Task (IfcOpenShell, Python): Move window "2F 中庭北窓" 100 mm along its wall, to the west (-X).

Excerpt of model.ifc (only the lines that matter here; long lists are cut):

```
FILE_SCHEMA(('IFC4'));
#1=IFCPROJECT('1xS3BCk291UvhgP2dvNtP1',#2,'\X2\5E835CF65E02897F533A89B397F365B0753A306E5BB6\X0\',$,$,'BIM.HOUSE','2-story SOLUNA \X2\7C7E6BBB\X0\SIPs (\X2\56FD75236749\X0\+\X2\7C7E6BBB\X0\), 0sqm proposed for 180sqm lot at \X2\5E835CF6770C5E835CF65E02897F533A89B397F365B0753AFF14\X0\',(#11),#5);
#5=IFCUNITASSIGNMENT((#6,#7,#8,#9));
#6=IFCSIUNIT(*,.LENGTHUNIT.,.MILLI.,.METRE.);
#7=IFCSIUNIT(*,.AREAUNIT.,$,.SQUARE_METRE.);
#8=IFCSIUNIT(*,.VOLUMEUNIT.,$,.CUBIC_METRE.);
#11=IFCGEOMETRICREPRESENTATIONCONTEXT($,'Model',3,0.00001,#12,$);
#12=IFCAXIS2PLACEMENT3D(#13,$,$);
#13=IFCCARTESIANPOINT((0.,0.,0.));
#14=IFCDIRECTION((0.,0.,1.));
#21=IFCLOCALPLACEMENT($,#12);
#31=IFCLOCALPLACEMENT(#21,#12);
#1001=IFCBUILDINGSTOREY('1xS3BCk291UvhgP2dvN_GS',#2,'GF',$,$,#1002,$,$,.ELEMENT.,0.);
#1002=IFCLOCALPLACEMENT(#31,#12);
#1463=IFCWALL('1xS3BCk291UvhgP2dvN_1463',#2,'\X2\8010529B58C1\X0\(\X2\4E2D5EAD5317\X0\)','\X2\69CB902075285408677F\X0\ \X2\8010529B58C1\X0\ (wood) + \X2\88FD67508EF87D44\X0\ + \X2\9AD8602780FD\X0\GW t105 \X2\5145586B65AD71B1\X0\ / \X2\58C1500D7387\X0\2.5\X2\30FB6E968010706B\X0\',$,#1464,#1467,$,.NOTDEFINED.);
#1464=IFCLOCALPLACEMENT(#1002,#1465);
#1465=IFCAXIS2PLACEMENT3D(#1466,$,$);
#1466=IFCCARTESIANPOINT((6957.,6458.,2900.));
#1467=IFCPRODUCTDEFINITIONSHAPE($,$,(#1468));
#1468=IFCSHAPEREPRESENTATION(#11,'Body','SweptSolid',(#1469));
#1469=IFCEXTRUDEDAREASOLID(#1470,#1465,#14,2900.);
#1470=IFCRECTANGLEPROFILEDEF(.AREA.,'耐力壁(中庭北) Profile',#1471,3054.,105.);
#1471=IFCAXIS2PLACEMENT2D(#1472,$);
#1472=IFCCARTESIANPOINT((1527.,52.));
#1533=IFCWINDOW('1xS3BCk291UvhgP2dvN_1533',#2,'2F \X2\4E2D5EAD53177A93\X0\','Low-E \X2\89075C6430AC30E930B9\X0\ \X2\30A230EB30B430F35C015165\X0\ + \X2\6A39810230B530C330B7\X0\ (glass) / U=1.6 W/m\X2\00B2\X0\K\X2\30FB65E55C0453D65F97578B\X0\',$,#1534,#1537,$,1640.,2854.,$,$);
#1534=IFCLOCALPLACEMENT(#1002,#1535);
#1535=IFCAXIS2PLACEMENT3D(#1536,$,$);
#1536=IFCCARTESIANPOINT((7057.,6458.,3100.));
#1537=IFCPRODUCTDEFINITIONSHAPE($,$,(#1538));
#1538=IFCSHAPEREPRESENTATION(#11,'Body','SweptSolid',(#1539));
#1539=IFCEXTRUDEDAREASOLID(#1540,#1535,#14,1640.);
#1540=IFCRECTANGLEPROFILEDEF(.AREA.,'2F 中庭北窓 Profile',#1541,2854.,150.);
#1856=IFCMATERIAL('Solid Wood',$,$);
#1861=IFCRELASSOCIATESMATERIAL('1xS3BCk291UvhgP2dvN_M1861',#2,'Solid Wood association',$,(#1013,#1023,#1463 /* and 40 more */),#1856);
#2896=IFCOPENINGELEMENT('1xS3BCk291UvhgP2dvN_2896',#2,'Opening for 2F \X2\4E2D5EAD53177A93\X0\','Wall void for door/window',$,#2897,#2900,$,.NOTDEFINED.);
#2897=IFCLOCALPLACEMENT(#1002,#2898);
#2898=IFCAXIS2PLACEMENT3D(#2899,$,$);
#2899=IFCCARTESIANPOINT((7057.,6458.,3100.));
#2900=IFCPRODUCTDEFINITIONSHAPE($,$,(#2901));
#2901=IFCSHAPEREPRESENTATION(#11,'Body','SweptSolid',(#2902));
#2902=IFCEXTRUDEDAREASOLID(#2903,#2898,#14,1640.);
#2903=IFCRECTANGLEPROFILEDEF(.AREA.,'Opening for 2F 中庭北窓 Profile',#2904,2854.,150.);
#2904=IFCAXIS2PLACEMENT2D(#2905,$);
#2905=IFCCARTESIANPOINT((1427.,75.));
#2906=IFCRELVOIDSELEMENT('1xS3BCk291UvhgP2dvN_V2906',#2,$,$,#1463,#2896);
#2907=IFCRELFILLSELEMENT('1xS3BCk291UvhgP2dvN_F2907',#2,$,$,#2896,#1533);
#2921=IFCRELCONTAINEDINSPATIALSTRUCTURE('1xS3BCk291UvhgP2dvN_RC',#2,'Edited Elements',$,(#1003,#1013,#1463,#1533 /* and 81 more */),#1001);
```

```python
import ifcopenshell
import ifcopenshell.api.geometry
import ifcopenshell.util.placement

model = ifcopenshell.open("model.ifc")

window = model.by_guid("1xS3BCk291UvhgP2dvN_1533")
opening = window.FillsVoids[0].RelatingOpeningElement
wall = opening.VoidsElements[0].RelatingBuildingElement

wall_matrix = ifcopenshell.util.placement.get_local_placement(wall.ObjectPlacement)
shift = wall_matrix[:3, 0] * -100.0
before = ifcopenshell.util.placement.get_local_placement(window.ObjectPlacement)[:3, 3].copy()

# The window is not placed relative to its opening, so move both.
for product in (opening, window):
    matrix = ifcopenshell.util.placement.get_local_placement(product.ObjectPlacement)
    matrix[:3, 3] += shift
    ifcopenshell.api.geometry.edit_object_placement(model, product=product, matrix=matrix, is_si=False)

after = ifcopenshell.util.placement.get_local_placement(window.ObjectPlacement)[:3, 3]
print("window moved by", (after - before).round(3) + 0.0)

model.write("model_v2.ifc")
```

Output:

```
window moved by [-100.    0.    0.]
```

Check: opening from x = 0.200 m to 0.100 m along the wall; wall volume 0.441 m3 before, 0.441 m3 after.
